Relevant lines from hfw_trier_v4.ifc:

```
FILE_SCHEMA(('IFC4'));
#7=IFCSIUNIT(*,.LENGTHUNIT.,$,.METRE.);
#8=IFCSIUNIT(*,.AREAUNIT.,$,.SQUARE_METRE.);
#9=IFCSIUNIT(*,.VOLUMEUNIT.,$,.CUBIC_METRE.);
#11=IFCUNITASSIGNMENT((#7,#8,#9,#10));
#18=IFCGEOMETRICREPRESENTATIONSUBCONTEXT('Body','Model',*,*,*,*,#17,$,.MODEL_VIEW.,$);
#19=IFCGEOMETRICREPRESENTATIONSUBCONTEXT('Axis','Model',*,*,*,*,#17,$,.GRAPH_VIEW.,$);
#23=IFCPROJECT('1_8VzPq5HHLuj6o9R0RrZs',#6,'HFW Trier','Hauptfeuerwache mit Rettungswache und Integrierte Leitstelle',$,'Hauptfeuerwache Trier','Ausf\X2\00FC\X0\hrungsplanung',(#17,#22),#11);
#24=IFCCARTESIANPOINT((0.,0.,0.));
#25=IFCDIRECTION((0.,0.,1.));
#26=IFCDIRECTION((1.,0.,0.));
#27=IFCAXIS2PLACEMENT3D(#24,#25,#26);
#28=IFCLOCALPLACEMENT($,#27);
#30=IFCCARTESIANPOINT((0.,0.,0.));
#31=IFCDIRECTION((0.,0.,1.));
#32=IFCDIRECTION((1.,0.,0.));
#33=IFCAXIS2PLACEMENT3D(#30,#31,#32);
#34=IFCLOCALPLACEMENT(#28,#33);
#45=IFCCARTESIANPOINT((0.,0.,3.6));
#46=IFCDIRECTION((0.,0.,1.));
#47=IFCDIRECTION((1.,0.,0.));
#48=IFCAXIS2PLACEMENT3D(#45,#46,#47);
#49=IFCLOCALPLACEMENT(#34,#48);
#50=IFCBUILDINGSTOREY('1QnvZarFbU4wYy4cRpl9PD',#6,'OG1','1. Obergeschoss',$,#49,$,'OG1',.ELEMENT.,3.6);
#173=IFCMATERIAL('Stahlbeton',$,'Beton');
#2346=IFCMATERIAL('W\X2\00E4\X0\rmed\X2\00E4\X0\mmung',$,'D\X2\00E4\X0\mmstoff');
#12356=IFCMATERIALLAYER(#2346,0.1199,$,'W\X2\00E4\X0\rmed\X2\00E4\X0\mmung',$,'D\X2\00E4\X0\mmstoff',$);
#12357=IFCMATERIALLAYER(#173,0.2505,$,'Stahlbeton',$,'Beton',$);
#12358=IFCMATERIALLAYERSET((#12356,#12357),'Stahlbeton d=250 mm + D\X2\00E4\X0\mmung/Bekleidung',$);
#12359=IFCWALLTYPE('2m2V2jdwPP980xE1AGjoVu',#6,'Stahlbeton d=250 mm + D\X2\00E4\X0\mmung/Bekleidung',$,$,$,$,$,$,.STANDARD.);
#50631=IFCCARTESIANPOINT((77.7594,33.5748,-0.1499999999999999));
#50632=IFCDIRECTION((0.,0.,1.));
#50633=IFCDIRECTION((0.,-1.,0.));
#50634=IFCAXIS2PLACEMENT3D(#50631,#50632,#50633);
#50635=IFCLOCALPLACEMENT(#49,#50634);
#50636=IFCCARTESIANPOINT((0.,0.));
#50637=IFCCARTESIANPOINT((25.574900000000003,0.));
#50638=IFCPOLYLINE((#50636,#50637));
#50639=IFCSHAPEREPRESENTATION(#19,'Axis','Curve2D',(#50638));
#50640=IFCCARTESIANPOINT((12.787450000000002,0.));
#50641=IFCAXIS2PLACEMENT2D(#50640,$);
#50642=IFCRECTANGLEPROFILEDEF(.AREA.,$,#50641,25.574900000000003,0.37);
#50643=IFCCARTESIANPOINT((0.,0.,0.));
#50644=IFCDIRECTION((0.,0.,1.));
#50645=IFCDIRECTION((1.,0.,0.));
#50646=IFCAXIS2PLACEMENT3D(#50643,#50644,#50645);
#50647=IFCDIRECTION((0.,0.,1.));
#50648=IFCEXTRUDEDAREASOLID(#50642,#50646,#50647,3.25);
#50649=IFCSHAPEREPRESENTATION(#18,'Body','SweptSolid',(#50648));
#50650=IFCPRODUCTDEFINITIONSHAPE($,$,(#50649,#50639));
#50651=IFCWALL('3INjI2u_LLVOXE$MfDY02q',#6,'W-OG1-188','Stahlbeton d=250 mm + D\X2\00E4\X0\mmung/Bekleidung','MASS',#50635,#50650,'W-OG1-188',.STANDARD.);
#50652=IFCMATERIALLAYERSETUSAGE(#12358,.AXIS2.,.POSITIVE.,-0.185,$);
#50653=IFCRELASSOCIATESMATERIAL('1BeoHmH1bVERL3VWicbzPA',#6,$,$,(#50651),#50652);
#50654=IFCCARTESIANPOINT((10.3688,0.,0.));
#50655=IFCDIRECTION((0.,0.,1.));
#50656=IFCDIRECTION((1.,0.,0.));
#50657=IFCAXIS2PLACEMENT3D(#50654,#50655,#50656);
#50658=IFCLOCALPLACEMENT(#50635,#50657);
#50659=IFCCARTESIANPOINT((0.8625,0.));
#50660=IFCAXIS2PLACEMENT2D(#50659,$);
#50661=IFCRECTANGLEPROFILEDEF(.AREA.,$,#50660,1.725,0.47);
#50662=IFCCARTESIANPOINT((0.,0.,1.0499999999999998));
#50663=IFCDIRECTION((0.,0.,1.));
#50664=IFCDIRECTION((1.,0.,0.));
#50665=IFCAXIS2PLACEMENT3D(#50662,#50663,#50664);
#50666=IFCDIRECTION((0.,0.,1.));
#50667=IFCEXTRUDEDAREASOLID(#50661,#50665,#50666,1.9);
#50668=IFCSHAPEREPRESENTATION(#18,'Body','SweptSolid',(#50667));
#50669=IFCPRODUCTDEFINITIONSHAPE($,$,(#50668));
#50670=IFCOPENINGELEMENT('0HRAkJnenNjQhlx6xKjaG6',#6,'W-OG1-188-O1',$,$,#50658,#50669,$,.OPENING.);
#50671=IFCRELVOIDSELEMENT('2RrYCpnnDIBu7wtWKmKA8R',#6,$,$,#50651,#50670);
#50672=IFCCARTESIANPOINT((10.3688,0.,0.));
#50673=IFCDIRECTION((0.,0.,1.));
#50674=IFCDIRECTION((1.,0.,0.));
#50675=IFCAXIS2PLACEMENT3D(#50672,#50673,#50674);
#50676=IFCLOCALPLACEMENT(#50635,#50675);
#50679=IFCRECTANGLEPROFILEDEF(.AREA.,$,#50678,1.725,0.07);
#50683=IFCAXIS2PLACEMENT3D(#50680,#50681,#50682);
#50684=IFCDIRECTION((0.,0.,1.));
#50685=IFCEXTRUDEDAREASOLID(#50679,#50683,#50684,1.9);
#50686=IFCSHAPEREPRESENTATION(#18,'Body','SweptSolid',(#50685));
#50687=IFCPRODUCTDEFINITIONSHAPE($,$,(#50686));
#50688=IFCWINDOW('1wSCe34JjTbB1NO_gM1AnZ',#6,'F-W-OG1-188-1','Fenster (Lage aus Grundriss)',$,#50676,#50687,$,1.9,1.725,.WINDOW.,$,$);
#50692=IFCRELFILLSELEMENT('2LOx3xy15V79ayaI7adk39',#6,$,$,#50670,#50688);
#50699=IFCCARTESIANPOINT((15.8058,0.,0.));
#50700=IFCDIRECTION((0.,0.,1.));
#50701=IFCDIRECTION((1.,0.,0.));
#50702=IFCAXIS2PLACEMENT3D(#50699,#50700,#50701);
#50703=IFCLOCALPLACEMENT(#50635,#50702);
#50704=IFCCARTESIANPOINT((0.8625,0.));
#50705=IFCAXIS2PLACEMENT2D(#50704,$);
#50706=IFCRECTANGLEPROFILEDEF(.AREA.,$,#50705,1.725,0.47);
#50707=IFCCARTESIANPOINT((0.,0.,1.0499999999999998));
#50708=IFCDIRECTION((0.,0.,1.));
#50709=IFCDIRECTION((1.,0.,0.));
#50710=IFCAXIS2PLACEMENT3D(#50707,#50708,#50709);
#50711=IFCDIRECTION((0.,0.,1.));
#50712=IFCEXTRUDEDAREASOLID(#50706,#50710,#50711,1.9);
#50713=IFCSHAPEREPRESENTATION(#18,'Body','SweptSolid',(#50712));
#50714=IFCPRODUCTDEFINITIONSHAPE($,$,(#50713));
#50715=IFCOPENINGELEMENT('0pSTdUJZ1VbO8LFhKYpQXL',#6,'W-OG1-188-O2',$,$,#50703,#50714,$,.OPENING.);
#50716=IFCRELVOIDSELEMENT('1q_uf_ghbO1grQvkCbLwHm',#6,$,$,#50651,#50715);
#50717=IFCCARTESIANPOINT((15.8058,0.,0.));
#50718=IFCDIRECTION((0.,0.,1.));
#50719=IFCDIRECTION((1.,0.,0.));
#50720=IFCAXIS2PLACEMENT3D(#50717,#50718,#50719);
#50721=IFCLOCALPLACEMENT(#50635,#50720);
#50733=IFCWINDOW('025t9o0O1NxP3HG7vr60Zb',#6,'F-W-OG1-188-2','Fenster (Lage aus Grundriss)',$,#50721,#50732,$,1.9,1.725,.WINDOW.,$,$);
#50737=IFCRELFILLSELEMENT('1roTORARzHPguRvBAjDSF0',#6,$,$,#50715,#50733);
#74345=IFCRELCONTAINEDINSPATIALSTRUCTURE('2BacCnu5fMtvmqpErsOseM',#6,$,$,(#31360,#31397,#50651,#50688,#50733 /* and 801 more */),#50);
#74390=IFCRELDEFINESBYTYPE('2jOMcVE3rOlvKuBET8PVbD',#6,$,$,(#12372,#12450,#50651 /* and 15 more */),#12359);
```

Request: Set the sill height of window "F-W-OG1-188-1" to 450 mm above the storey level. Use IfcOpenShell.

```python
import numpy as np
import ifcopenshell
import ifcopenshell.api.geometry
import ifcopenshell.geom
import ifcopenshell.util.element
import ifcopenshell.util.placement
import ifcopenshell.util.shape
import ifcopenshell.util.unit

model = ifcopenshell.open("hfw_trier_v4.ifc")
unit_scale = ifcopenshell.util.unit.calculate_unit_scale(model)

window = model.by_guid("1wSCe34JjTbB1NO_gM1AnZ")
opening = window.FillsVoids[0].RelatingOpeningElement
storey = ifcopenshell.util.element.get_container(window, ifc_class="IfcBuildingStorey")
level = ifcopenshell.util.placement.get_local_placement(storey.ObjectPlacement)[2, 3]

# The opening's origin need not be at the sill, so measure its lowest point.
shape = ifcopenshell.geom.create_shape(ifcopenshell.geom.settings(), opening)
bottom = ifcopenshell.util.shape.get_shape_bottom_elevation(shape, shape.geometry) / unit_scale
dz = level + 0.45 - bottom

shift = np.array([0.0, 0.0, dz])
# The window is not placed relative to its opening, so move both.
for product in (opening, window):
    matrix = ifcopenshell.util.placement.get_local_placement(product.ObjectPlacement)
    matrix[:3, 3] += shift
    ifcopenshell.api.geometry.edit_object_placement(model, product=product, matrix=matrix, is_si=False)

print(f"moved by {dz * unit_scale:+.3f} m")

model.write("hfw_trier_v4_updated.ifc")
```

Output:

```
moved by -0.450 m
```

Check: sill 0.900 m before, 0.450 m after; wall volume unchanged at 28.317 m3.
